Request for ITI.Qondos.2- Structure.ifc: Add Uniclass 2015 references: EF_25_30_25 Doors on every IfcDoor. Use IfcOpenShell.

First a look at what the model holds.

```python
import ifcopenshell

model = ifcopenshell.open("ITI.Qondos.2- Structure.ifc")
print(model.schema)
print("classifications:", [c.Name for c in model.by_type("IfcClassification")])
for ifc_class in ("IfcDoor", "IfcRoof", "IfcStair", "IfcWall", "IfcWindow"):
    print(ifc_class, len(model.by_type(ifc_class)))
```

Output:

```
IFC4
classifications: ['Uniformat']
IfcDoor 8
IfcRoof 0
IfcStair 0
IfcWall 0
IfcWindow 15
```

```python
import ifcopenshell
import ifcopenshell.api.classification

model = ifcopenshell.open("ITI.Qondos.2- Structure.ifc")

system = ifcopenshell.api.classification.add_classification(model, classification="Uniclass 2015")

codes = {
    "IfcDoor": ("EF_25_30_25", "Doors"),
}
for ifc_class, (code, name) in codes.items():
    products = model.by_type(ifc_class)
    ifcopenshell.api.classification.add_reference(
        model, products=products, classification=system, identification=code, name=name
    )
    print(code, len(products))

model.write("ITI.Qondos.2- Structure_edited.ifc")
```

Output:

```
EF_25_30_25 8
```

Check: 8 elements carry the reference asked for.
